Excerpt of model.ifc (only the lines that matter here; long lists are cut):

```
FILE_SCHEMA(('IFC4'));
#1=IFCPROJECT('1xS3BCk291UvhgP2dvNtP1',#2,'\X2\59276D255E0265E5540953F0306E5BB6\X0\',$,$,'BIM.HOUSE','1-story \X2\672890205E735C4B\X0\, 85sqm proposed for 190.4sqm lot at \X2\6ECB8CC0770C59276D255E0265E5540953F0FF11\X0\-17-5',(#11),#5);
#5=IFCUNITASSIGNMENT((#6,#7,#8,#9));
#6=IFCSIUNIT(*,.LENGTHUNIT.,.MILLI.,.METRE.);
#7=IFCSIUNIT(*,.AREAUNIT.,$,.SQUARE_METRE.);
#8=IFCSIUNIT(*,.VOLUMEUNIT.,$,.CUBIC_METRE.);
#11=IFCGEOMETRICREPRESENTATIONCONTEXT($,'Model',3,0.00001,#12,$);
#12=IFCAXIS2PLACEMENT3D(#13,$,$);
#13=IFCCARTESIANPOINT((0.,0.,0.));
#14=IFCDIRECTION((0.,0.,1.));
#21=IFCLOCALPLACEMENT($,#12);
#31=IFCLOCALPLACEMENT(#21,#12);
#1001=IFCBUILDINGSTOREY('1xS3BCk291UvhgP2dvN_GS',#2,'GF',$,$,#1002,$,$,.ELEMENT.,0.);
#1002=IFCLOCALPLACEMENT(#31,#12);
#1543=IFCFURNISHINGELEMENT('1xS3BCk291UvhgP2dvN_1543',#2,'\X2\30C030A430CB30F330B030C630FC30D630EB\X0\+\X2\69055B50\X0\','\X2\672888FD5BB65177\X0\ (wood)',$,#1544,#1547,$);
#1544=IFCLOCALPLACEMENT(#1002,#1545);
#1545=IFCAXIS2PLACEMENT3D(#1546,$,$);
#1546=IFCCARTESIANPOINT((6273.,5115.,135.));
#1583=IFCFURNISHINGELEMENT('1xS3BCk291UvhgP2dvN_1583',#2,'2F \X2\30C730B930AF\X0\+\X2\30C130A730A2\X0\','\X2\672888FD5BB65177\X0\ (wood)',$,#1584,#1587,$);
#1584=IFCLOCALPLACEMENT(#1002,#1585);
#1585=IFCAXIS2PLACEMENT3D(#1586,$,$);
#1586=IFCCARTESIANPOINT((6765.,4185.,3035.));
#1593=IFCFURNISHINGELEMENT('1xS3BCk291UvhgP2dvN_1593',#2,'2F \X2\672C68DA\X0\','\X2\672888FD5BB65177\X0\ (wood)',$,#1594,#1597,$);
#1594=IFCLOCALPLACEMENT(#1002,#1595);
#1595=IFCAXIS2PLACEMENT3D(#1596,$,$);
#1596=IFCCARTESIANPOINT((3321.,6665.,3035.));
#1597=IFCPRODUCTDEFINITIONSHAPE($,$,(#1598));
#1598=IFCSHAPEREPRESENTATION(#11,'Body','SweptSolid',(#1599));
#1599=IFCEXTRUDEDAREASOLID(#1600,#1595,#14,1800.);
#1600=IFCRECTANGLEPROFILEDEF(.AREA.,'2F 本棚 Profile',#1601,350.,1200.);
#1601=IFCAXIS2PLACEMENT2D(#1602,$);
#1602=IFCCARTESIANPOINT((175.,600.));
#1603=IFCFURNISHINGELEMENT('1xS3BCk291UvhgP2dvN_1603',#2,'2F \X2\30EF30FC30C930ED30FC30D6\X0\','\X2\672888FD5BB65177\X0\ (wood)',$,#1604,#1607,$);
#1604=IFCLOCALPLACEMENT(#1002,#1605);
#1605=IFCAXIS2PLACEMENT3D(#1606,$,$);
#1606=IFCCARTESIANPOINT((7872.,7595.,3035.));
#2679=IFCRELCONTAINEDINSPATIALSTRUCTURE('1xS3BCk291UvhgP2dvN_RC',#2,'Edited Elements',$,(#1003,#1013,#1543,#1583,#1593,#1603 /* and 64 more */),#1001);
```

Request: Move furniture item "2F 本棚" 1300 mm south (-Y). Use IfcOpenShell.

```python
import ifcopenshell
import ifcopenshell.api.geometry
import ifcopenshell.util.placement
import ifcopenshell.util.unit

model = ifcopenshell.open("model.ifc")
unit_scale = ifcopenshell.util.unit.calculate_unit_scale(model)

item = model.by_guid("1xS3BCk291UvhgP2dvN_1593")
matrix = ifcopenshell.util.placement.get_local_placement(item.ObjectPlacement)
matrix[1, 3] -= 1.3 / unit_scale
ifcopenshell.api.geometry.edit_object_placement(model, product=item, matrix=matrix, is_si=False)

print(ifcopenshell.util.placement.get_local_placement(item.ObjectPlacement).round(3) + 0.0)

model.write("model-out.ifc")
```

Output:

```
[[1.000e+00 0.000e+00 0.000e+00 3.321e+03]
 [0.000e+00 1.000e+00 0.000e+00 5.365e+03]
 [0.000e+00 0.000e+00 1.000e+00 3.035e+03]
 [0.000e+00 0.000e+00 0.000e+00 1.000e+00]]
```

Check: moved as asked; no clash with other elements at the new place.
